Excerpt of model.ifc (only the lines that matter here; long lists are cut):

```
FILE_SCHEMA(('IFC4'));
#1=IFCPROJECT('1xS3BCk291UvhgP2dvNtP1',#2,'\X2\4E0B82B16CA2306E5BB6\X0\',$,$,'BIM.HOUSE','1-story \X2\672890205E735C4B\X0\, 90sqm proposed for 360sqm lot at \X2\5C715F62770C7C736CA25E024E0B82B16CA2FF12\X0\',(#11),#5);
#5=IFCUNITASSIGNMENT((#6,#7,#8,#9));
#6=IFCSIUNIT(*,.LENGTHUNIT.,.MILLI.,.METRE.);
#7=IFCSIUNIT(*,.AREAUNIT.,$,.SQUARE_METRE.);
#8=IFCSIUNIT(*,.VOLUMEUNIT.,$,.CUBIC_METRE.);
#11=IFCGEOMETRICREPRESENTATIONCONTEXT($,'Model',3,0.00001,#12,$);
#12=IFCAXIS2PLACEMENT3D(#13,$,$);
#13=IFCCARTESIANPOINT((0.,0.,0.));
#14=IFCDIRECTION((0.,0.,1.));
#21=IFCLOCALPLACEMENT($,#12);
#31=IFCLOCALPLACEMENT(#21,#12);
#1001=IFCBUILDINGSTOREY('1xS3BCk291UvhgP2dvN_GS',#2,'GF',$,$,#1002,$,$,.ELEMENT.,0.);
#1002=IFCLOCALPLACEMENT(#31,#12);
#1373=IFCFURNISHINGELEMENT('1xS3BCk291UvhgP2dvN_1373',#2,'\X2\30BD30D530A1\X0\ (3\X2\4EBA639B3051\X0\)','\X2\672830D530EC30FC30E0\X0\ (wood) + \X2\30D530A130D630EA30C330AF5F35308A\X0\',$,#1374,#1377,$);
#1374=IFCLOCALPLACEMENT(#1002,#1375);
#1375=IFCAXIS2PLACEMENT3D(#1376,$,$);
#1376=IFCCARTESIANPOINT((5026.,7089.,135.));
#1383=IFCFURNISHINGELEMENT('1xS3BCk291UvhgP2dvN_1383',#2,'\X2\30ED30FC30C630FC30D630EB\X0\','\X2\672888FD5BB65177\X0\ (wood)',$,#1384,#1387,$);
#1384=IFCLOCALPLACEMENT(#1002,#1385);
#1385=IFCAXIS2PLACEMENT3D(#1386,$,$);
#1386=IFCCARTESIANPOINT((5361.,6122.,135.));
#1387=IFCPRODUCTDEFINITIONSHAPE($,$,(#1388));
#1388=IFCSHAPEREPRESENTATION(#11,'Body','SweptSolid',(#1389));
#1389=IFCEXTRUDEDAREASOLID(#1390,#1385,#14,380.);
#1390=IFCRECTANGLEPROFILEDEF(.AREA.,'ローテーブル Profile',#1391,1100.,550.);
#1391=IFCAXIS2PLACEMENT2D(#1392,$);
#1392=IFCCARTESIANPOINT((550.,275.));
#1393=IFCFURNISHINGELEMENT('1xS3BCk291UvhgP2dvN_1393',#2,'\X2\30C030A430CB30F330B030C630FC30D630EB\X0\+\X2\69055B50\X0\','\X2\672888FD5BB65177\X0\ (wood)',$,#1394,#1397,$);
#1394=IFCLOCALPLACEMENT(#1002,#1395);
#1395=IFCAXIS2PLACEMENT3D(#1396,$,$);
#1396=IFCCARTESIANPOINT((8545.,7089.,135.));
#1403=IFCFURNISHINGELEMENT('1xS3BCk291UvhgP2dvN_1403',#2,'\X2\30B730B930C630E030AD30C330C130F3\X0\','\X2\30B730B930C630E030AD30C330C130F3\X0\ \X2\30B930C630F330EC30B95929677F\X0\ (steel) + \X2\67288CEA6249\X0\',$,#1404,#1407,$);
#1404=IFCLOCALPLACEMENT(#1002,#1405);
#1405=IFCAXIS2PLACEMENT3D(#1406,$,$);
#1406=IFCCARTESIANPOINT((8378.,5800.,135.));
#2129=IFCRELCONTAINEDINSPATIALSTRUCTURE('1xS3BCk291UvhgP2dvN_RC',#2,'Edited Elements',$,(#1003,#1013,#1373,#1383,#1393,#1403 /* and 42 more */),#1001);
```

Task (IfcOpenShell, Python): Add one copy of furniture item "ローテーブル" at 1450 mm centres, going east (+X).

```python
import numpy as np
import ifcopenshell
import ifcopenshell.api.geometry
import ifcopenshell.api.root
import ifcopenshell.util.element
import ifcopenshell.util.placement
import ifcopenshell.util.unit

model = ifcopenshell.open("model.ifc")
unit_scale = ifcopenshell.util.unit.calculate_unit_scale(model)


def reuse_history(source, copy):
    """copy_class also copies each property set's owner history, people and application; keep the originals."""
    for rel in copy.IsDefinedBy:
        if rel.is_a("IfcRelDefinesByProperties") and (history := rel.RelatingPropertyDefinition.OwnerHistory):
            rel.RelatingPropertyDefinition.OwnerHistory = source.OwnerHistory
            ifcopenshell.util.element.remove_deep2(model, history)


source = model.by_guid("1xS3BCk291UvhgP2dvN_1383")
base = ifcopenshell.util.placement.get_local_placement(source.ObjectPlacement)
step = np.array([1.0, 0.0, 0.0]) * 1.45 / unit_scale

for i in range(1, 2):
    copy = ifcopenshell.api.root.copy_class(model, product=source)
    copy.Representation = ifcopenshell.util.element.copy_deep(
        model, source.Representation, exclude=["IfcGeometricRepresentationContext", "IfcRepresentationMap"]
    )
    reuse_history(source, copy)
    matrix = base.copy()
    matrix[:3, 3] += i * step
    print("added at", matrix[:3, 3].round(3) + 0.0)
    ifcopenshell.api.geometry.edit_object_placement(model, product=copy, matrix=matrix, is_si=False)

model.write("model_edited.ifc")
```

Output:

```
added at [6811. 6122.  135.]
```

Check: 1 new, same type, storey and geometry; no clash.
